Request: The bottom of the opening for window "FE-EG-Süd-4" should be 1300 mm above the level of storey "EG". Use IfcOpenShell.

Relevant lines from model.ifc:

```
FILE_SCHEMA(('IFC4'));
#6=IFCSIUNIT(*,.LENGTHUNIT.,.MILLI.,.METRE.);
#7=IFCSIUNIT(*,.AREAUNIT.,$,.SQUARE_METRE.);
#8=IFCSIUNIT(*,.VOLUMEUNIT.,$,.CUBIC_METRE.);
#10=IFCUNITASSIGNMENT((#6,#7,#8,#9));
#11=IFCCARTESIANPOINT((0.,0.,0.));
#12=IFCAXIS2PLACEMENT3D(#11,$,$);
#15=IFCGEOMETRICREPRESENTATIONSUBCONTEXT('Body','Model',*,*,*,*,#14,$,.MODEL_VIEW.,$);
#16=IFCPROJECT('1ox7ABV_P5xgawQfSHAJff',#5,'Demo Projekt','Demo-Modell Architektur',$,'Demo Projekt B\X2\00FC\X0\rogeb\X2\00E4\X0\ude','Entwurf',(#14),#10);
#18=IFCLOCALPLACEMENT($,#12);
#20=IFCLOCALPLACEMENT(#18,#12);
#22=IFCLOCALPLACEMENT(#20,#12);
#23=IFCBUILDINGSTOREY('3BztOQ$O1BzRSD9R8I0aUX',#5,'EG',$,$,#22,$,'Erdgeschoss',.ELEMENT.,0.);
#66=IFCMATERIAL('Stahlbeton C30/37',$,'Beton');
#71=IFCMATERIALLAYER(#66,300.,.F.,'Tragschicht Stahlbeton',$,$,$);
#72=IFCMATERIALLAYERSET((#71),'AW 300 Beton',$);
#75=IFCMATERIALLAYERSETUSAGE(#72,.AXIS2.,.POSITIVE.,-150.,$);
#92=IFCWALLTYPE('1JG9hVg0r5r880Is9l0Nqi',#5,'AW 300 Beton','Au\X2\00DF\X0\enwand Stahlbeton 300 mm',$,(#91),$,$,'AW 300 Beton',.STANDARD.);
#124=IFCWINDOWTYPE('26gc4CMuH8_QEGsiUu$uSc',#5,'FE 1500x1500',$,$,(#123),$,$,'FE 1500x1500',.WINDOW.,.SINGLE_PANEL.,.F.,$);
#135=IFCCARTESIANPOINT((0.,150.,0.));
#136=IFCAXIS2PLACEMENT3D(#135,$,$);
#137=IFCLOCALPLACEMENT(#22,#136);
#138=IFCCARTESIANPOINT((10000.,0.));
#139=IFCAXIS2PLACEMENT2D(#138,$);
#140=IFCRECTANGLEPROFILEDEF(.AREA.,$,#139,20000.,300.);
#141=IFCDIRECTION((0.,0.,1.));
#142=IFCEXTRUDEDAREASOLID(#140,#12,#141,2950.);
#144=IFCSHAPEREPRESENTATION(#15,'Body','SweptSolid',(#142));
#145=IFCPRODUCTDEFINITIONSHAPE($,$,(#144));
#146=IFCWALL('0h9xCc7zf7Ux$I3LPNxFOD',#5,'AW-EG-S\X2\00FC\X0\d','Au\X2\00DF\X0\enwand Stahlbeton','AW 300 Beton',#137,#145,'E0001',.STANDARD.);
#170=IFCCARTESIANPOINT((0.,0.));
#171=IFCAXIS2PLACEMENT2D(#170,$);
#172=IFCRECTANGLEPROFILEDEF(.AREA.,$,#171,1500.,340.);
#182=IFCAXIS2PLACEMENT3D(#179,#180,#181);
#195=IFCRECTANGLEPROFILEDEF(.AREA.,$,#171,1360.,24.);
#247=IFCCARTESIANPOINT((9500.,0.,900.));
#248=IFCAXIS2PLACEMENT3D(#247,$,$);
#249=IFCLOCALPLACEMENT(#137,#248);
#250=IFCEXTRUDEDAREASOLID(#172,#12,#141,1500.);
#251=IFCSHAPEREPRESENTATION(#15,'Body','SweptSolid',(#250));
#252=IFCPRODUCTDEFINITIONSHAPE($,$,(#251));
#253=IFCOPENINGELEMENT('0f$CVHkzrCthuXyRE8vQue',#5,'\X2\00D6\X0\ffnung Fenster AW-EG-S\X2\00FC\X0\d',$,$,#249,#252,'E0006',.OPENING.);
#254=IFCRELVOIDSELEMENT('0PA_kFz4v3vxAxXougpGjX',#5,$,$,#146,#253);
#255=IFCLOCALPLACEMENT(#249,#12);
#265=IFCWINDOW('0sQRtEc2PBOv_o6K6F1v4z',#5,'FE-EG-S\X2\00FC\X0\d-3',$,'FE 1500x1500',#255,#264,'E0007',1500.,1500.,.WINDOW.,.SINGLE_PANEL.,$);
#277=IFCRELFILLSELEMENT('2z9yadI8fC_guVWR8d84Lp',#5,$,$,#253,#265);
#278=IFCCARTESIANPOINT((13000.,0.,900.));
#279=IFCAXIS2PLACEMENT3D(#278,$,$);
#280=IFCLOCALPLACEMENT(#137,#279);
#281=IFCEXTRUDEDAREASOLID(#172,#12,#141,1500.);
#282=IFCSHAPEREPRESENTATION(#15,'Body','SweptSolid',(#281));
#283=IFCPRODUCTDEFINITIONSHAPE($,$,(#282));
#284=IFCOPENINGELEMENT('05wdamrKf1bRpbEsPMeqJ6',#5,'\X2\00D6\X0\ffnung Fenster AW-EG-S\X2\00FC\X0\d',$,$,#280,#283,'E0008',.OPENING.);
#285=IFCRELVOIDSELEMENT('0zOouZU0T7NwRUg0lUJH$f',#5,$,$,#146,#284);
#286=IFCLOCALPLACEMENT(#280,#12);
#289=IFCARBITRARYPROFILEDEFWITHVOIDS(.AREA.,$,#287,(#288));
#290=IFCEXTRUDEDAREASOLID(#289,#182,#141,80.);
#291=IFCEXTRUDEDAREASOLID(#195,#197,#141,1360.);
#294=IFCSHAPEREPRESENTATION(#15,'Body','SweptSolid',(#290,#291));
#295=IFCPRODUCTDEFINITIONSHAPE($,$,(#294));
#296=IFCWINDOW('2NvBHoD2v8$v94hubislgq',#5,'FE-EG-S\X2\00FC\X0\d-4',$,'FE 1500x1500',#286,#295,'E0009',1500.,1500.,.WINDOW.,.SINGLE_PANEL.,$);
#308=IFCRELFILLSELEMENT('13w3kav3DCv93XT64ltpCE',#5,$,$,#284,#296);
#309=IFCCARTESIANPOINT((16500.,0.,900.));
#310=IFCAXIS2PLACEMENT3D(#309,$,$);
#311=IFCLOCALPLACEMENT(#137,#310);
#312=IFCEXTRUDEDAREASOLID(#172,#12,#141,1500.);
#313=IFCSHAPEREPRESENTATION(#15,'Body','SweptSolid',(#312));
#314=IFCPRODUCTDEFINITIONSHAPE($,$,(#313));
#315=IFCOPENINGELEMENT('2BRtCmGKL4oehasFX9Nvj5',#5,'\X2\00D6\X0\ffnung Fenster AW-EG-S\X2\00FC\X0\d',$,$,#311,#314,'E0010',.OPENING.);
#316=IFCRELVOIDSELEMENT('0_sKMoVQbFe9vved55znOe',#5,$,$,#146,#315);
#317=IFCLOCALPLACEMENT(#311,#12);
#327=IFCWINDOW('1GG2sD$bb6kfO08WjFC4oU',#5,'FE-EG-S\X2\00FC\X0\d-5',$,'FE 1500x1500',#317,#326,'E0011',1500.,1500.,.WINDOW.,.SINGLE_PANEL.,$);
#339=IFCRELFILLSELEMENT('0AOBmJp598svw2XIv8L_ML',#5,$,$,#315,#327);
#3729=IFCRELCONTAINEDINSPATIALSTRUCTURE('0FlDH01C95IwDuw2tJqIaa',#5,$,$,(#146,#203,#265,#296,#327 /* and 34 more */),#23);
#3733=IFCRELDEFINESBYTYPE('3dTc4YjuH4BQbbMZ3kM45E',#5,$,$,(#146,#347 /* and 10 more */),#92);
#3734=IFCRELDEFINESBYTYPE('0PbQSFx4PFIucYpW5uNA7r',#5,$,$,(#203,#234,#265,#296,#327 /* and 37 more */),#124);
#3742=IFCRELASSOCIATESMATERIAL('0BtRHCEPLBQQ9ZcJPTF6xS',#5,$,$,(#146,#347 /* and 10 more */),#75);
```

```python
import numpy as np
import ifcopenshell
import ifcopenshell.api.geometry
import ifcopenshell.geom
import ifcopenshell.util.element
import ifcopenshell.util.placement
import ifcopenshell.util.shape
import ifcopenshell.util.unit

model = ifcopenshell.open("model.ifc")
unit_scale = ifcopenshell.util.unit.calculate_unit_scale(model)

window = model.by_guid("2NvBHoD2v8$v94hubislgq")
opening = window.FillsVoids[0].RelatingOpeningElement
storey = ifcopenshell.util.element.get_container(window, ifc_class="IfcBuildingStorey")
level = ifcopenshell.util.placement.get_local_placement(storey.ObjectPlacement)[2, 3]

# The opening's origin need not be at the sill, so measure its lowest point.
shape = ifcopenshell.geom.create_shape(ifcopenshell.geom.settings(), opening)
bottom = ifcopenshell.util.shape.get_shape_bottom_elevation(shape, shape.geometry) / unit_scale
dz = level + 1300.0 - bottom

shift = np.array([0.0, 0.0, dz])
# The window is placed relative to its opening, so it follows when the opening moves.
matrix = ifcopenshell.util.placement.get_local_placement(opening.ObjectPlacement)
matrix[:3, 3] += shift
ifcopenshell.api.geometry.edit_object_placement(
    model, product=opening, matrix=matrix, is_si=False, should_transform_children=True
)

print(f"moved by {dz * unit_scale:+.3f} m")

model.write("model_rev.ifc")
```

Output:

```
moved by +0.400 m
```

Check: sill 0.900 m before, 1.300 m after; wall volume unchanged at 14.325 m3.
